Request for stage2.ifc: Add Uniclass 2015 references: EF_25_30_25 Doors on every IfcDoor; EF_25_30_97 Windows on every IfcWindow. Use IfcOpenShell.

First a look at what the model holds.

```python
import ifcopenshell

model = ifcopenshell.open("stage2.ifc")
print(model.schema)
print("classifications:", [c.Name for c in model.by_type("IfcClassification")])
for ifc_class in ("IfcDoor", "IfcRoof", "IfcStair", "IfcWall", "IfcWindow"):
    print(ifc_class, len(model.by_type(ifc_class)))
```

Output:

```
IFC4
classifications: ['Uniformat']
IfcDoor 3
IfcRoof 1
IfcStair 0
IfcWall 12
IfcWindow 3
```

```python
import ifcopenshell
import ifcopenshell.api.classification

model = ifcopenshell.open("stage2.ifc")

system = ifcopenshell.api.classification.add_classification(model, classification="Uniclass 2015")

codes = {
    "IfcDoor": ("EF_25_30_25", "Doors"),
    "IfcWindow": ("EF_25_30_97", "Windows"),
}
for ifc_class, (code, name) in codes.items():
    products = model.by_type(ifc_class)
    ifcopenshell.api.classification.add_reference(
        model, products=products, classification=system, identification=code, name=name
    )
    print(code, len(products))

model.write("stage2_edited.ifc")
```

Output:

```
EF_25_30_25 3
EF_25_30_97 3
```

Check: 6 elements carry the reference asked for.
